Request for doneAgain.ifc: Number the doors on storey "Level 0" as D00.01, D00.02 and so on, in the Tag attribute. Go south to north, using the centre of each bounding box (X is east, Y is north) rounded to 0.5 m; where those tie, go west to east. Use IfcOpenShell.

First a look at what the model holds.

```python
import ifcopenshell
import ifcopenshell.util.element
import ifcopenshell.util.placement

model = ifcopenshell.open("doneAgain.ifc")
print(model.schema)
storey = next(s for s in model.by_type("IfcBuildingStorey") if s.Name == "Level 0")
doors = [e for e in ifcopenshell.util.element.get_decomposition(storey) if e.is_a("IfcDoor")]
for e in sorted(doors, key=lambda e: e.id()):
    origin = ifcopenshell.util.placement.get_local_placement(e.ObjectPlacement)[:3, 3]
    print(e.id(), e.Tag, e.Name, origin.round(2) + 0.0, sep=" | ")
```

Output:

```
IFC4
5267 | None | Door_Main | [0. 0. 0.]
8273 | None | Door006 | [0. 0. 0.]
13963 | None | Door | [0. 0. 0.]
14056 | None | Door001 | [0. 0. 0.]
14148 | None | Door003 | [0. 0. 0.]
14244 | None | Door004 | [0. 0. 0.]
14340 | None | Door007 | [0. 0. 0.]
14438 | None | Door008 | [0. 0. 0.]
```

```python
import ifcopenshell
import ifcopenshell.geom
import ifcopenshell.util.element
import ifcopenshell.util.shape

model = ifcopenshell.open("doneAgain.ifc")
settings = ifcopenshell.geom.settings()
settings.set("use-world-coords", True)


def centre(element):
    shape = ifcopenshell.geom.create_shape(settings, element)
    return ifcopenshell.util.shape.get_bbox_centroid(shape.geometry)


storey = next(s for s in model.by_type("IfcBuildingStorey") if s.Name == "Level 0")
doors = [e for e in ifcopenshell.util.element.get_decomposition(storey) if e.is_a("IfcDoor")]

# Insertion points can sit at a corner or the storey origin, so sort by the geometry (in metres).
centres = {e: centre(e) for e in doors}
doors.sort(key=lambda e: (round(centres[e][1] / 0.5), centres[e][0]))

for i, e in enumerate(doors, start=1):
    number = f"D00.{i:02d}"
    e.Tag = number
    print(e.id(), number)

model.write("doneAgain_rev.ifc")
```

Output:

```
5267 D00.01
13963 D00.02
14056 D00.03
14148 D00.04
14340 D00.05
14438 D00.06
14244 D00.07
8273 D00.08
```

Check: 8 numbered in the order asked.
